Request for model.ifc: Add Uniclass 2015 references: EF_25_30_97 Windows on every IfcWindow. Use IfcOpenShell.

First a look at what the model holds.

```python
import ifcopenshell

model = ifcopenshell.open("model.ifc")
print(model.schema)
print("classifications:", [c.Name for c in model.by_type("IfcClassification")])
for ifc_class in ("IfcDoor", "IfcRoof", "IfcStair", "IfcWall", "IfcWindow"):
    print(ifc_class, len(model.by_type(ifc_class)))
```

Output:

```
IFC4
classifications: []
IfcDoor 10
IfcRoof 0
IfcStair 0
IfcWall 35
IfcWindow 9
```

```python
import ifcopenshell
import ifcopenshell.api.classification

model = ifcopenshell.open("model.ifc")

system = ifcopenshell.api.classification.add_classification(model, classification="Uniclass 2015")

codes = {
    "IfcWindow": ("EF_25_30_97", "Windows"),
}
for ifc_class, (code, name) in codes.items():
    products = model.by_type(ifc_class)
    ifcopenshell.api.classification.add_reference(
        model, products=products, classification=system, identification=code, name=name
    )
    print(code, len(products))

model.write("model_rev.ifc")
```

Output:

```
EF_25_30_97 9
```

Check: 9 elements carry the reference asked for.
